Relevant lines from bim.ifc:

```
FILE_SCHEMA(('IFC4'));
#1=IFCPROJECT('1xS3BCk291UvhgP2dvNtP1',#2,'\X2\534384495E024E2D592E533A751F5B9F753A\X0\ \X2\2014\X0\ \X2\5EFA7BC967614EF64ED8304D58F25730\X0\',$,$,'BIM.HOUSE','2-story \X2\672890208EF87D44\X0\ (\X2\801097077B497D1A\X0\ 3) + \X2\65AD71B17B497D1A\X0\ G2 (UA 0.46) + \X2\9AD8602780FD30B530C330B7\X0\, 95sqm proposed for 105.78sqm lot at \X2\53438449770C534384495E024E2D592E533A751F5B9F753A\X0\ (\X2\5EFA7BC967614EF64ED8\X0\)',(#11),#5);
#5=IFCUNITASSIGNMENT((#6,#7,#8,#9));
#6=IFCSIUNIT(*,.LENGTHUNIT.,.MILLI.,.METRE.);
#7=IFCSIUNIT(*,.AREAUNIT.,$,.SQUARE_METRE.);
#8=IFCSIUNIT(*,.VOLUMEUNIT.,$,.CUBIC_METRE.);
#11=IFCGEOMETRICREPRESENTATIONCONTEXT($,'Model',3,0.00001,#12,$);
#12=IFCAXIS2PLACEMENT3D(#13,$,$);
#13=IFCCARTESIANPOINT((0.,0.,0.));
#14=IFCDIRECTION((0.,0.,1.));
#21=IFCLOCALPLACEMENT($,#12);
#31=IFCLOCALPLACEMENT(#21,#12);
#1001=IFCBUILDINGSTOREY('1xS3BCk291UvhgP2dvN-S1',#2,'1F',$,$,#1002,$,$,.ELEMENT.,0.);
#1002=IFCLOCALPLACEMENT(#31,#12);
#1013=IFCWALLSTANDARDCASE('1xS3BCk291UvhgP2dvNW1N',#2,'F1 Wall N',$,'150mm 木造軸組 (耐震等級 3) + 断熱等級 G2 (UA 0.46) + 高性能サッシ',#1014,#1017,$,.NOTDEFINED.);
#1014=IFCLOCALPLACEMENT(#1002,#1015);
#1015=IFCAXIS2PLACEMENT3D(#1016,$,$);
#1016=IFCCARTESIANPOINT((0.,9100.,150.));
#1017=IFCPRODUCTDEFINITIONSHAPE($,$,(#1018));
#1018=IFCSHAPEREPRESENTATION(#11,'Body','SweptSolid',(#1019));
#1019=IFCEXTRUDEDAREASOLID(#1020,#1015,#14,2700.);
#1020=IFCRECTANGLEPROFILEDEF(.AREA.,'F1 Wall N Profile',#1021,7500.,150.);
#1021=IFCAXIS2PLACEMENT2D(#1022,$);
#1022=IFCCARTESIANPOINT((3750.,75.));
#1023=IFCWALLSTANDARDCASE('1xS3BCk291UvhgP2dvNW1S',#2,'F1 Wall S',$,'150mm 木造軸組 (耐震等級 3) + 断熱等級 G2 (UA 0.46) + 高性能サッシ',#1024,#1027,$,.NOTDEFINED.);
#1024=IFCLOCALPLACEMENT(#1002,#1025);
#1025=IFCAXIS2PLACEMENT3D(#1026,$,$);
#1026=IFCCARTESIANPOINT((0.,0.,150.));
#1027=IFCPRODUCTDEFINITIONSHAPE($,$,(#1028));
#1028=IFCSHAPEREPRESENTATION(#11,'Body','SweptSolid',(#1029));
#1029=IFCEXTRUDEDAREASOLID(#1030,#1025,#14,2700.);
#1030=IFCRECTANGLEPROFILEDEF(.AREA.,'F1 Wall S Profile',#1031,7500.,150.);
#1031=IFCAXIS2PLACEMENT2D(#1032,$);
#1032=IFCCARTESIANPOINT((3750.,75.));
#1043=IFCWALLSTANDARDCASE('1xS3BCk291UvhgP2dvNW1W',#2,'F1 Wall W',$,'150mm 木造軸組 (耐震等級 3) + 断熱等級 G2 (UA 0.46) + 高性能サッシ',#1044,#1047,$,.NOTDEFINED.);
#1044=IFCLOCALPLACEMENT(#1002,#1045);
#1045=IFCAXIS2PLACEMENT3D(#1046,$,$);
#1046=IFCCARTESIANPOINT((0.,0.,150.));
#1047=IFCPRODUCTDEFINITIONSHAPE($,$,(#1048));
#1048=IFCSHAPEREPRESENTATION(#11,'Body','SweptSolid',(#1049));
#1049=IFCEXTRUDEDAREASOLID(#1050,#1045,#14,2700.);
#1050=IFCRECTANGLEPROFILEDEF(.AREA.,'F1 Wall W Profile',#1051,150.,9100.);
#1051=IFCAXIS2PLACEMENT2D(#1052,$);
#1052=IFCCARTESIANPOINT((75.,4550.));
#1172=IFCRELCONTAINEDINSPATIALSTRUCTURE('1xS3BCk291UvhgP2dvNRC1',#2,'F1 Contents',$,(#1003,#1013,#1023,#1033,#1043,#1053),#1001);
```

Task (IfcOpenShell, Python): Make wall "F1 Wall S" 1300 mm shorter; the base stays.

```python
import ifcopenshell
import ifcopenshell.geom
import ifcopenshell.util.shape
import ifcopenshell.util.unit

model = ifcopenshell.open("bim.ifc")
unit_scale = ifcopenshell.util.unit.calculate_unit_scale(model)
settings = ifcopenshell.geom.settings()


def volume(element):
    """Net volume in cubic metres, openings subtracted."""
    shape = ifcopenshell.geom.create_shape(settings, element)
    return ifcopenshell.util.shape.get_volume(shape.geometry)


wall = model.by_guid("1xS3BCk291UvhgP2dvNW1S")
before = volume(wall)

body = next(r for r in wall.Representation.Representations if r.RepresentationIdentifier == "Body")
solid = body.Items[0]
old_height = solid.Depth
solid.Depth -= 1.3 / unit_scale
after = volume(wall)

print(f"height {old_height:g} -> {solid.Depth:g}, volume {before:.3f} -> {after:.3f} m3")

model.write("bim_v2.ifc")
```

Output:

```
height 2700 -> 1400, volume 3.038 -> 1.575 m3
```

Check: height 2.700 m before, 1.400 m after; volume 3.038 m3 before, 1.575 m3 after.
